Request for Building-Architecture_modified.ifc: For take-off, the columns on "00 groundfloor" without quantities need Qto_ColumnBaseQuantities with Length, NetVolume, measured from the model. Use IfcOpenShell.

First a look at what the model holds.

```python
import ifcopenshell
import ifcopenshell.util.element
import ifcopenshell.util.unit

model = ifcopenshell.open("Building-Architecture_modified.ifc")
print(model.schema)
for unit_type in ("LENGTHUNIT", "AREAUNIT", "VOLUMEUNIT"):
    print(unit_type, ifcopenshell.util.unit.calculate_unit_scale(model, unit_type))
storey = next(s for s in model.by_type("IfcBuildingStorey") if s.Name == "00 groundfloor")
columns = [e for e in ifcopenshell.util.element.get_decomposition(storey) if e.is_a("IfcColumn")]
for e in sorted(columns, key=lambda e: e.id()):
    print(e.id(), e.is_a(), e.Name, list(ifcopenshell.util.element.get_psets(e, qtos_only=True)), sep=" | ")
```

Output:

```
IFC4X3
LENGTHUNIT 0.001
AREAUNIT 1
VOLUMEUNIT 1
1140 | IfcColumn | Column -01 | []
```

```python
import ifcopenshell
import ifcopenshell.api.pset
import ifcopenshell.geom
import ifcopenshell.util.element
import ifcopenshell.util.shape
import ifcopenshell.util.unit

model = ifcopenshell.open("Building-Architecture_modified.ifc")
unit_scale = ifcopenshell.util.unit.calculate_unit_scale(model)
volume_scale = ifcopenshell.util.unit.calculate_unit_scale(model, "VOLUMEUNIT")
settings = ifcopenshell.geom.settings()

storey = next(s for s in model.by_type("IfcBuildingStorey") if s.Name == "00 groundfloor")
columns = [e for e in ifcopenshell.util.element.get_decomposition(storey) if e.is_a("IfcColumn")]

for e in sorted(columns, key=lambda e: e.id()):
    if ifcopenshell.util.element.get_psets(e, qtos_only=True, should_inherit=False):
        continue
    # Geometry comes back in metres, in the element's own axes.
    shape = ifcopenshell.geom.create_shape(settings, e)
    values = {
        "Length": ifcopenshell.util.shape.get_z(shape.geometry) / unit_scale,
        "NetVolume": ifcopenshell.util.shape.get_volume(shape.geometry) / volume_scale,
    }
    qto = ifcopenshell.api.pset.add_qto(model, product=e, name="Qto_ColumnBaseQuantities")
    ifcopenshell.api.pset.edit_qto(model, qto=qto, properties=values)
    print(e.id(), {k: round(v, 3) for k, v in values.items()})

model.write("Building-Architecture_modified_v2.ifc")
```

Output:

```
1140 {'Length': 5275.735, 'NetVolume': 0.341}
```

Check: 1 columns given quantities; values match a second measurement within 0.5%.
